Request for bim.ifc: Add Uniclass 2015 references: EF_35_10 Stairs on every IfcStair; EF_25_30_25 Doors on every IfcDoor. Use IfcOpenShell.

First a look at what the model holds.

```python
import ifcopenshell

model = ifcopenshell.open("bim.ifc")
print(model.schema)
print("classifications:", [c.Name for c in model.by_type("IfcClassification")])
for ifc_class in ("IfcDoor", "IfcRoof", "IfcStair", "IfcWall", "IfcWindow"):
    print(ifc_class, len(model.by_type(ifc_class)))
```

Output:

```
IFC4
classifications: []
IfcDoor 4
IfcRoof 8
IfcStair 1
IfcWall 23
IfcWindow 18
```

```python
import ifcopenshell
import ifcopenshell.api.classification

model = ifcopenshell.open("bim.ifc")

system = ifcopenshell.api.classification.add_classification(model, classification="Uniclass 2015")

codes = {
    "IfcStair": ("EF_35_10", "Stairs"),
    "IfcDoor": ("EF_25_30_25", "Doors"),
}
for ifc_class, (code, name) in codes.items():
    products = model.by_type(ifc_class)
    ifcopenshell.api.classification.add_reference(
        model, products=products, classification=system, identification=code, name=name
    )
    print(code, len(products))

model.write("bim_edited.ifc")
```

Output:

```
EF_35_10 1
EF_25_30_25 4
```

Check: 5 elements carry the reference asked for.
